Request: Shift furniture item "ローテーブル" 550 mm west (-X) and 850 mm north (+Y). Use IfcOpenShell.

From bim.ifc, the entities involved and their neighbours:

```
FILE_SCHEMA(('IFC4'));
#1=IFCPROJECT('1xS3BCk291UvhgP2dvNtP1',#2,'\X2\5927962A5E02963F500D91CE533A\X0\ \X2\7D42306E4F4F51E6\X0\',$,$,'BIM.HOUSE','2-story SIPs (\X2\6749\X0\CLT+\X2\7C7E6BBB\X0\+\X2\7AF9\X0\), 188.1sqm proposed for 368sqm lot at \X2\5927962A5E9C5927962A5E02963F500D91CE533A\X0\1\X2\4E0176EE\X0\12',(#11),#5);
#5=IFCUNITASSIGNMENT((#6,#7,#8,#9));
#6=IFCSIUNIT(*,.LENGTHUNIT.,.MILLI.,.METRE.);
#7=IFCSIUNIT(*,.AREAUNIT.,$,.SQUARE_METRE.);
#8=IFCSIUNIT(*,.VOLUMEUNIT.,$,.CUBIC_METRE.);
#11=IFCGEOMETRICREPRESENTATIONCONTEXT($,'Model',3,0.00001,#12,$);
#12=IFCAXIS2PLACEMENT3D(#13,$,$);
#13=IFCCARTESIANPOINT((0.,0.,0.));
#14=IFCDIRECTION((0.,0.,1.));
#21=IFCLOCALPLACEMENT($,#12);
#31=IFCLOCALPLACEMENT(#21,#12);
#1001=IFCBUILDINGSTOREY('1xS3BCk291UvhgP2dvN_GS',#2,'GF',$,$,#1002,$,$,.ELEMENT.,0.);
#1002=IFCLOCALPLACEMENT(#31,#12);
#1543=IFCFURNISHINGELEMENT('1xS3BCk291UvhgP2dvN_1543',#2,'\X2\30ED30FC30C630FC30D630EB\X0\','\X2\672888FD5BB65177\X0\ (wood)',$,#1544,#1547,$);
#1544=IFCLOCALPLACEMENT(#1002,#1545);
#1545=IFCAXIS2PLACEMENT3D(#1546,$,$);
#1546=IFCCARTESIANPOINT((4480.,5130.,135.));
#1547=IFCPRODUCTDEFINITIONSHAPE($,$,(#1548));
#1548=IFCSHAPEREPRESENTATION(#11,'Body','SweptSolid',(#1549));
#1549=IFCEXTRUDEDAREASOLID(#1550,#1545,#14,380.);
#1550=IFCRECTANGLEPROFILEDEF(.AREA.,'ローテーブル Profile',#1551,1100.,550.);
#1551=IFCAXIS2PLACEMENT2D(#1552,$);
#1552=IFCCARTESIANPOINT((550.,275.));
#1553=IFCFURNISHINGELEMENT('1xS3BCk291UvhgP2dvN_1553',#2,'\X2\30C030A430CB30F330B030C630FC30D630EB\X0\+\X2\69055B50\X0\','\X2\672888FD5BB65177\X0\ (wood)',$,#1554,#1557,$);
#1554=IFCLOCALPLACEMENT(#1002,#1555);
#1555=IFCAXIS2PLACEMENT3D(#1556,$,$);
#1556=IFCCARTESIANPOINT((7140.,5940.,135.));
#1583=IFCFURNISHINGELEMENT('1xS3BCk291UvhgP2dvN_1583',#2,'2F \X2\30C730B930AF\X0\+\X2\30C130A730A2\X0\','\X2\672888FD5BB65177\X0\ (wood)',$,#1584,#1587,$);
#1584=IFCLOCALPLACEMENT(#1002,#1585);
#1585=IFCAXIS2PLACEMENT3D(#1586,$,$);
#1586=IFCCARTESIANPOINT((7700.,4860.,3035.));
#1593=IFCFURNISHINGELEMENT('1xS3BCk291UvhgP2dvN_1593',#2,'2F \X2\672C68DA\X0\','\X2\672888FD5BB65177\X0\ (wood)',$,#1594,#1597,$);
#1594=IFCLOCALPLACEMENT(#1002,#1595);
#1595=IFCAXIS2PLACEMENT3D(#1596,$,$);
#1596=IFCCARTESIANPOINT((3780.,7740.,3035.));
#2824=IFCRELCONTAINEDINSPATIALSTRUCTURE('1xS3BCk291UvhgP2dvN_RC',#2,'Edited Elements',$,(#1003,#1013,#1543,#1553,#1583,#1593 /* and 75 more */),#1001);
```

```python
import ifcopenshell
import ifcopenshell.api.geometry
import ifcopenshell.util.placement
import ifcopenshell.util.unit

model = ifcopenshell.open("bim.ifc")
unit_scale = ifcopenshell.util.unit.calculate_unit_scale(model)

item = model.by_guid("1xS3BCk291UvhgP2dvN_1543")
matrix = ifcopenshell.util.placement.get_local_placement(item.ObjectPlacement)
matrix[0, 3] -= 0.55 / unit_scale
matrix[1, 3] += 0.85 / unit_scale
ifcopenshell.api.geometry.edit_object_placement(model, product=item, matrix=matrix, is_si=False)

print(ifcopenshell.util.placement.get_local_placement(item.ObjectPlacement).round(3) + 0.0)

model.write("bim_v2.ifc")
```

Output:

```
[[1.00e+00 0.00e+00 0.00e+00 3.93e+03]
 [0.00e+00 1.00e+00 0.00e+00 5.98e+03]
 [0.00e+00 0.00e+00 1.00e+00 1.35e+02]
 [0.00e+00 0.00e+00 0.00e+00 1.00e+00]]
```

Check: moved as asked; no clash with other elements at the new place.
